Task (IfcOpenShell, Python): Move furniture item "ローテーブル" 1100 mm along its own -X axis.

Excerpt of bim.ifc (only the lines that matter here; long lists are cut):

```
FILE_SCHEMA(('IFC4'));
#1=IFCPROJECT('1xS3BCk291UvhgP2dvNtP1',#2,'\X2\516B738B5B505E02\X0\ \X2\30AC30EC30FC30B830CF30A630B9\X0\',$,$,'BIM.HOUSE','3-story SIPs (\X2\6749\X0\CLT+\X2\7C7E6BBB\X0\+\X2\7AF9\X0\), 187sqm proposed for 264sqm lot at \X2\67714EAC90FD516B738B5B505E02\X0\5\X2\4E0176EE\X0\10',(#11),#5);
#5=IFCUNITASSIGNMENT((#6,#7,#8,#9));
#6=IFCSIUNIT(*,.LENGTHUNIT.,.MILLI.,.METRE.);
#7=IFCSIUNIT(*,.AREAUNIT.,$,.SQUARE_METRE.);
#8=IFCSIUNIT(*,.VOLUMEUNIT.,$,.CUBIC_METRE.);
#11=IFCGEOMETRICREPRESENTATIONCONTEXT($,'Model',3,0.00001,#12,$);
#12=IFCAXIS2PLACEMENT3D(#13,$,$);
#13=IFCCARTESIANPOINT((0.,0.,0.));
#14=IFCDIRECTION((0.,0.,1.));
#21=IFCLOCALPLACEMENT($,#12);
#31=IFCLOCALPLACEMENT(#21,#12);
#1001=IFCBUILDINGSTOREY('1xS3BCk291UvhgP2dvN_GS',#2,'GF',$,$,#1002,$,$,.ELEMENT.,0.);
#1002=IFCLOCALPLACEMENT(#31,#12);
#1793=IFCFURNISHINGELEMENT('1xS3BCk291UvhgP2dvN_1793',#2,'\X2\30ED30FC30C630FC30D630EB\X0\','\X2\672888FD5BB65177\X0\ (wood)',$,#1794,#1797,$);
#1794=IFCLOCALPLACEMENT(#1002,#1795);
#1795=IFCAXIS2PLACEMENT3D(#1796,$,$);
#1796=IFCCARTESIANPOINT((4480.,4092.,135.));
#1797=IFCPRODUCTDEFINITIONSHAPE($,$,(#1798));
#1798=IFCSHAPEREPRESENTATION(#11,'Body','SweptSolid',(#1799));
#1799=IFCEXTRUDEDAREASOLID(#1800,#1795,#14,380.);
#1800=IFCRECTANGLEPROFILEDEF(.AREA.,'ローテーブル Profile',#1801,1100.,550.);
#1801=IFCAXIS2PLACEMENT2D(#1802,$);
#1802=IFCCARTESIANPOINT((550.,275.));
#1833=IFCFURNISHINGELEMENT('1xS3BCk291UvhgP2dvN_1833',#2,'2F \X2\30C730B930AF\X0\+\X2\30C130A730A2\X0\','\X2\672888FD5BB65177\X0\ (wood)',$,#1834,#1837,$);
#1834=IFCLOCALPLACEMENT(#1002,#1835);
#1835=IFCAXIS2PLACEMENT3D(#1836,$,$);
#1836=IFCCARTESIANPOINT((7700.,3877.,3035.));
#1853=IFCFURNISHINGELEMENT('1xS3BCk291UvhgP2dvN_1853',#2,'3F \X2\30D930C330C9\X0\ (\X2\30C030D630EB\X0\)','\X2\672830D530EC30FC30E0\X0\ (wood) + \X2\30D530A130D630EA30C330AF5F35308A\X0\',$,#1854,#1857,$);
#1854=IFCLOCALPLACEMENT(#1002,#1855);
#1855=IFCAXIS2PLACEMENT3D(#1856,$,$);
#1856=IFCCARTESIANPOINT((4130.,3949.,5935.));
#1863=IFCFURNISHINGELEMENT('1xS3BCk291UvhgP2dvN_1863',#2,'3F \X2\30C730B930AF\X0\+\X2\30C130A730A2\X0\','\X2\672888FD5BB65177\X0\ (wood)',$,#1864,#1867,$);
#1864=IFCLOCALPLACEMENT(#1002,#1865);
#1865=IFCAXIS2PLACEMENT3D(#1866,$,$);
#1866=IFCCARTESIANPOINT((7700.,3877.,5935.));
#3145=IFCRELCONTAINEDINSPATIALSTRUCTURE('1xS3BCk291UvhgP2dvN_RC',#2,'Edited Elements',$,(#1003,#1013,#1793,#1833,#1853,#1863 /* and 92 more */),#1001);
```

```python
import ifcopenshell
import ifcopenshell.api.geometry
import ifcopenshell.util.placement
import ifcopenshell.util.unit

model = ifcopenshell.open("bim.ifc")
unit_scale = ifcopenshell.util.unit.calculate_unit_scale(model)

item = model.by_id(1793)
matrix = ifcopenshell.util.placement.get_local_placement(item.ObjectPlacement)
matrix[:3, 3] -= matrix[:3, 0] * 1.1 / unit_scale
ifcopenshell.api.geometry.edit_object_placement(model, product=item, matrix=matrix, is_si=False)

print(ifcopenshell.util.placement.get_local_placement(item.ObjectPlacement).round(3) + 0.0)

model.write("bim_updated.ifc")
```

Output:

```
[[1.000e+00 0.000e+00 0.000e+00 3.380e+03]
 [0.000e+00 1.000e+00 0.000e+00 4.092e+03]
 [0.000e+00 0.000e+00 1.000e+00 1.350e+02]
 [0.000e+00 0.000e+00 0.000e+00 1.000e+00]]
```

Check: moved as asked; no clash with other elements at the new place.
